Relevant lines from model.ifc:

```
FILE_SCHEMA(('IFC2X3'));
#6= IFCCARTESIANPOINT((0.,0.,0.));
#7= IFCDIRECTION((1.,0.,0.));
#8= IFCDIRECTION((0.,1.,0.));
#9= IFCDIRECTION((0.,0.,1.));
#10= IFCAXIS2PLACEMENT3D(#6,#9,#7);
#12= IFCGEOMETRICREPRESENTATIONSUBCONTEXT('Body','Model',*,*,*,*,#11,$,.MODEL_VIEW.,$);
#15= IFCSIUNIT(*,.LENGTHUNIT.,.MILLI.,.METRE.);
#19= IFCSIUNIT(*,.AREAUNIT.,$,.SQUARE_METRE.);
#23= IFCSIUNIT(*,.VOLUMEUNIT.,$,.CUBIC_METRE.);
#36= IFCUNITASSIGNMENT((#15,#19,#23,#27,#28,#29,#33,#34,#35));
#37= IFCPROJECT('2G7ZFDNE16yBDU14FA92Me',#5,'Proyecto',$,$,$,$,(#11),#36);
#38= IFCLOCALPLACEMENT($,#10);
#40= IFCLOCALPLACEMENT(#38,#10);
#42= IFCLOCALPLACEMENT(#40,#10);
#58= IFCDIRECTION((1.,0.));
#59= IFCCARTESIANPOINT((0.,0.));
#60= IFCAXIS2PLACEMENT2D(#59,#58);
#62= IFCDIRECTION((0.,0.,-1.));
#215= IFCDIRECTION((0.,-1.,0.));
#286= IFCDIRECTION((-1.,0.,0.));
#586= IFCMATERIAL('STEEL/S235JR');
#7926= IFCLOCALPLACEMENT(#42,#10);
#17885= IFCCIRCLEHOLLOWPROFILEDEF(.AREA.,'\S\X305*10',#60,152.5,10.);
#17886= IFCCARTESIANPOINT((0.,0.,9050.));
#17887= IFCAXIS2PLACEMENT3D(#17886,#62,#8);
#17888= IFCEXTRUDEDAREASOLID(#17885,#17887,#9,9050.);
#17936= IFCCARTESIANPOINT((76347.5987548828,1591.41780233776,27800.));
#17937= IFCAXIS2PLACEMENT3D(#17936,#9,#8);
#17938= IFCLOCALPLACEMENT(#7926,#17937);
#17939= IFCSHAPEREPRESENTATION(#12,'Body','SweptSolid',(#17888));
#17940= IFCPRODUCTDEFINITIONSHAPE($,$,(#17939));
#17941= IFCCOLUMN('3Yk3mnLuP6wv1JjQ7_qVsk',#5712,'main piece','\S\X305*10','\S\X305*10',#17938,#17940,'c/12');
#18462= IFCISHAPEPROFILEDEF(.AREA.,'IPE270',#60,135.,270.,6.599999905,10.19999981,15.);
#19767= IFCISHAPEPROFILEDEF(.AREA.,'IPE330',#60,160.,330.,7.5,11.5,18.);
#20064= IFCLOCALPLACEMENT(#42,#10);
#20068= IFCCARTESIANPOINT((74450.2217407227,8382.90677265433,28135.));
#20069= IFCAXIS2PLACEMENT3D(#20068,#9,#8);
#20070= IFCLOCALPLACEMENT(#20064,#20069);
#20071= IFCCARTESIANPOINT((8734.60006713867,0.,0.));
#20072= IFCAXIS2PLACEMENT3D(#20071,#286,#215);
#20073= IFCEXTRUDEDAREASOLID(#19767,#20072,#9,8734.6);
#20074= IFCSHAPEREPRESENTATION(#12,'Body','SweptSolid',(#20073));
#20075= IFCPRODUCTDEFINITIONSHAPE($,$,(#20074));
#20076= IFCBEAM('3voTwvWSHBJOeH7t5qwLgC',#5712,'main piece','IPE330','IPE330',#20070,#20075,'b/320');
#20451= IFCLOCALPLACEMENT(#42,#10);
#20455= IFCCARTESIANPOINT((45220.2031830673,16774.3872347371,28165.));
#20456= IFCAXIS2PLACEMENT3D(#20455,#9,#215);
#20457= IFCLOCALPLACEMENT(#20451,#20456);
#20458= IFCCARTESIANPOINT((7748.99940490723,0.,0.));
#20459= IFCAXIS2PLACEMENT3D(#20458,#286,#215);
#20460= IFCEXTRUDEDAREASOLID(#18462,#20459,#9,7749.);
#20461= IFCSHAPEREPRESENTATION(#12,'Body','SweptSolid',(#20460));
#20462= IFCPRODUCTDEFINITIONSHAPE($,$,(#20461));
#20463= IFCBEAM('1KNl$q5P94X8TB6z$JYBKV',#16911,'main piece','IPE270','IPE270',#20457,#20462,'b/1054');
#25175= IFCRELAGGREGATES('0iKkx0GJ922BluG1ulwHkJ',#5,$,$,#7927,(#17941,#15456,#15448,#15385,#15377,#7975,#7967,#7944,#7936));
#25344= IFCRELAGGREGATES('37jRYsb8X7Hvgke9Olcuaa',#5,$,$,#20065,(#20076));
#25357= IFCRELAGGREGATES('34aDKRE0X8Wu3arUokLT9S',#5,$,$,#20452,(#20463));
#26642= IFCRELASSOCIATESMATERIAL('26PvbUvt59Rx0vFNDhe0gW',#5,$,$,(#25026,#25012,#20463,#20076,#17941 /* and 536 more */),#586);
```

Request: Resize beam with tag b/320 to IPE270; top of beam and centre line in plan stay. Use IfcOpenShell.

```python
import ifcopenshell
import ifcopenshell.util.element
import ifcopenshell.util.representation

model = ifcopenshell.open("model.ifc")

member = model.by_guid("3voTwvWSHBJOeH7t5qwLgC")
source = next(p for p in model.by_type("IfcIShapeProfileDef") if p.ProfileName == "IPE270")

body = ifcopenshell.util.representation.get_representation(member, "Model", "Body")
solid = body.Items[0]
old_profile = solid.SweptArea

# Copy the section's sizes but keep this member's own profile position.
profile = ifcopenshell.util.element.copy(model, source)
# Profiles are centred, so shift by half the change in depth to hold the top.
shift = (old_profile.OverallDepth - profile.OverallDepth) / 2
x, y = old_profile.Position.Location.Coordinates
up = (0.0, 1.0)  # upwards, in the solid's own plane
location = model.createIfcCartesianPoint((x + up[0] * shift, y + up[1] * shift))
profile.Position = model.createIfcAxis2Placement2D(location, old_profile.Position.RefDirection)
solid.SweptArea = profile
if not model.get_total_inverses(old_profile):
    ifcopenshell.util.element.remove_deep2(model, old_profile)
member.Description = member.Description.replace("IPE330", "IPE270")
member.ObjectType = member.ObjectType.replace("IPE330", "IPE270")

print(solid.SweptArea)

model.write("model-out.ifc")
```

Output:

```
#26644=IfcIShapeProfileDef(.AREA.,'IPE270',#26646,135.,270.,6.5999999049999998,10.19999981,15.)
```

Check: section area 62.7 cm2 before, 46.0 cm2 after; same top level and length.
